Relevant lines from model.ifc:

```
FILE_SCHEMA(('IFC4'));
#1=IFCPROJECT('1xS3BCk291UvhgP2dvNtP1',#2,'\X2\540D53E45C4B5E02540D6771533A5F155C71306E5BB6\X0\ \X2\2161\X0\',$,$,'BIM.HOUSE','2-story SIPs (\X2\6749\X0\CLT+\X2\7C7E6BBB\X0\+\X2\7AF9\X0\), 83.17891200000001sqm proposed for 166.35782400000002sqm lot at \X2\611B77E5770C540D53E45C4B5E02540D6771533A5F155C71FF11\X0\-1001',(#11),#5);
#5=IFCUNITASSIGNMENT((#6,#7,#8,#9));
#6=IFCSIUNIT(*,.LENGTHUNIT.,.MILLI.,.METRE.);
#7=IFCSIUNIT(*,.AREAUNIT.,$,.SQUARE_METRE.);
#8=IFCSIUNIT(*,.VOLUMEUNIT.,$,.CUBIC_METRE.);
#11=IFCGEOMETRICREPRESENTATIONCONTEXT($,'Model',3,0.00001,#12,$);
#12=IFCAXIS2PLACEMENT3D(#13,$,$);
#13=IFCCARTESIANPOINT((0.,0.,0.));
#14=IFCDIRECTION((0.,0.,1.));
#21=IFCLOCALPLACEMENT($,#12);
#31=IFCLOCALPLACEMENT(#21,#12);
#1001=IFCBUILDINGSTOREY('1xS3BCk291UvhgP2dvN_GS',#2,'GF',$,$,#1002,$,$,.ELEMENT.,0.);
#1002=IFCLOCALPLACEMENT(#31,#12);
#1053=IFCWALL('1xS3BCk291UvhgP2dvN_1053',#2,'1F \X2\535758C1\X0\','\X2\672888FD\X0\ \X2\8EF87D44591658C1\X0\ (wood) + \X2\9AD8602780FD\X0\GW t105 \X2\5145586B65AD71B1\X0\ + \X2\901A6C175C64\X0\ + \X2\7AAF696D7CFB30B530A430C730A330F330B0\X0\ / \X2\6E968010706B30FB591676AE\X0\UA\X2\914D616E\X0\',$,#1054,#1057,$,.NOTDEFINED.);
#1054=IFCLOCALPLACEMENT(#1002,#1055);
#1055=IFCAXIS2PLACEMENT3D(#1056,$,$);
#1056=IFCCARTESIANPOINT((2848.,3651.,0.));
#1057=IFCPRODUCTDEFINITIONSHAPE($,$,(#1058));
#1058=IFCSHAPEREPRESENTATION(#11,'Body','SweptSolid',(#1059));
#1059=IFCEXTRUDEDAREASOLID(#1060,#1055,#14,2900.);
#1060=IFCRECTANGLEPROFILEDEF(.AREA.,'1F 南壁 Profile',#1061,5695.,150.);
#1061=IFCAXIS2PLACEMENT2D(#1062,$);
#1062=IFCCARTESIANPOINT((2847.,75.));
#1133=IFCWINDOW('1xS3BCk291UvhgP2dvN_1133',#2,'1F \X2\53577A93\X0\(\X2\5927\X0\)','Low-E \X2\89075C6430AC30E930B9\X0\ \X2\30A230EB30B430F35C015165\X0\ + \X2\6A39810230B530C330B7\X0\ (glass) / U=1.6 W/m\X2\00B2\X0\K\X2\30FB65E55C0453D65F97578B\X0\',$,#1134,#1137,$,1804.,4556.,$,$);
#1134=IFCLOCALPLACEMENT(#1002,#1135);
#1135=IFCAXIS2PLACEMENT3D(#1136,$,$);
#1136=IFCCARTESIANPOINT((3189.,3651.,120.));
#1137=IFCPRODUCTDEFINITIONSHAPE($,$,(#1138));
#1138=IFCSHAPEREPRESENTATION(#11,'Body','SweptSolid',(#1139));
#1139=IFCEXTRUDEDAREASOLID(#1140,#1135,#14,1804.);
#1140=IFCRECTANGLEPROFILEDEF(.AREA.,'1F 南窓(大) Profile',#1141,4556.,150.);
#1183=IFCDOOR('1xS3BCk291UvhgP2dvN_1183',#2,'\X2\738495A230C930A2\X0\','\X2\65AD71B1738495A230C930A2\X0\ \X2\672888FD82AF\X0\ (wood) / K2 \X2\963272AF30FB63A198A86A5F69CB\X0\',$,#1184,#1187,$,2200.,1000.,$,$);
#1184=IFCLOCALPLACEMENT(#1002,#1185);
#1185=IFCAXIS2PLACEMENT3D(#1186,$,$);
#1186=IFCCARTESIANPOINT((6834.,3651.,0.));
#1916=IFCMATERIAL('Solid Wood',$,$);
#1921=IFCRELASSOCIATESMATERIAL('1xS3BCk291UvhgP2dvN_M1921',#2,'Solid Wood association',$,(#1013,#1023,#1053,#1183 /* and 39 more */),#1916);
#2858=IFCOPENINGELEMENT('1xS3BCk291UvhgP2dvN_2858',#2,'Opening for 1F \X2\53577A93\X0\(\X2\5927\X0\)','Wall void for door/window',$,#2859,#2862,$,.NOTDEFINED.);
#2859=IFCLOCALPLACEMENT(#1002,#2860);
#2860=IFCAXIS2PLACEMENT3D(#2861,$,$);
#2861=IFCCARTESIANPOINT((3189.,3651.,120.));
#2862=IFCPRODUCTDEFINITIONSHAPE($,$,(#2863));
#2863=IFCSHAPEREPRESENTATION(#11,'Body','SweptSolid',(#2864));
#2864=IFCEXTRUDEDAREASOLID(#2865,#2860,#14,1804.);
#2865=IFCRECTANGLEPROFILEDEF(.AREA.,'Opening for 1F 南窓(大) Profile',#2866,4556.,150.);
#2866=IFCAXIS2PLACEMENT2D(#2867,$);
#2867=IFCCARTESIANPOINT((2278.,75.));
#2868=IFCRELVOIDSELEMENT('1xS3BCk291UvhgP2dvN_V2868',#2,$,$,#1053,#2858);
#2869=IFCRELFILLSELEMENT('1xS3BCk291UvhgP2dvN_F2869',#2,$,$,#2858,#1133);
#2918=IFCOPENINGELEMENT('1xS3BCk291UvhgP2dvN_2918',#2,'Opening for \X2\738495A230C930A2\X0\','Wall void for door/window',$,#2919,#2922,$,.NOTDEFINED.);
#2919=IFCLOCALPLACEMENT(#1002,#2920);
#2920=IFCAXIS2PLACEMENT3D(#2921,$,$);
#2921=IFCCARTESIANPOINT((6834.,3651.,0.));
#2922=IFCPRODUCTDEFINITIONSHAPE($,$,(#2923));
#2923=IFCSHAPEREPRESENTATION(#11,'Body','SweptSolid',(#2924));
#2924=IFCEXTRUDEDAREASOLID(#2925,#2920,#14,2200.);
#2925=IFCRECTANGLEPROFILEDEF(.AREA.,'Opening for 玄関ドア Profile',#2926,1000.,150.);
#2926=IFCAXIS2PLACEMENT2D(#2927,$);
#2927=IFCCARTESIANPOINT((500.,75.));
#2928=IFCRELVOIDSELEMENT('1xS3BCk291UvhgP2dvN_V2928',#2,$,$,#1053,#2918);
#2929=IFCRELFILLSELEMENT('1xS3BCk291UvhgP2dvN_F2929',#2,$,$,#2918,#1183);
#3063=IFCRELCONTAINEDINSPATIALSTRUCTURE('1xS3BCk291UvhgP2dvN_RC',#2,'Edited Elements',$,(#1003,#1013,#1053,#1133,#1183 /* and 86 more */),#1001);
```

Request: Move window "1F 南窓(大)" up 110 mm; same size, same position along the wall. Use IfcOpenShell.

```python
import numpy as np
import ifcopenshell
import ifcopenshell.api.geometry
import ifcopenshell.util.placement
import ifcopenshell.util.unit

model = ifcopenshell.open("model.ifc")
unit_scale = ifcopenshell.util.unit.calculate_unit_scale(model)

window = model.by_guid("1xS3BCk291UvhgP2dvN_1133")
opening = window.FillsVoids[0].RelatingOpeningElement
dz = 110.0

shift = np.array([0.0, 0.0, dz])
# The window is not placed relative to its opening, so move both.
for product in (opening, window):
    matrix = ifcopenshell.util.placement.get_local_placement(product.ObjectPlacement)
    matrix[:3, 3] += shift
    ifcopenshell.api.geometry.edit_object_placement(model, product=product, matrix=matrix, is_si=False)

print(f"moved by {dz * unit_scale:+.3f} m")

model.write("model_v2.ifc")
```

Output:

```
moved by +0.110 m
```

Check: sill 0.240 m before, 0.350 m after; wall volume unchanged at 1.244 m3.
